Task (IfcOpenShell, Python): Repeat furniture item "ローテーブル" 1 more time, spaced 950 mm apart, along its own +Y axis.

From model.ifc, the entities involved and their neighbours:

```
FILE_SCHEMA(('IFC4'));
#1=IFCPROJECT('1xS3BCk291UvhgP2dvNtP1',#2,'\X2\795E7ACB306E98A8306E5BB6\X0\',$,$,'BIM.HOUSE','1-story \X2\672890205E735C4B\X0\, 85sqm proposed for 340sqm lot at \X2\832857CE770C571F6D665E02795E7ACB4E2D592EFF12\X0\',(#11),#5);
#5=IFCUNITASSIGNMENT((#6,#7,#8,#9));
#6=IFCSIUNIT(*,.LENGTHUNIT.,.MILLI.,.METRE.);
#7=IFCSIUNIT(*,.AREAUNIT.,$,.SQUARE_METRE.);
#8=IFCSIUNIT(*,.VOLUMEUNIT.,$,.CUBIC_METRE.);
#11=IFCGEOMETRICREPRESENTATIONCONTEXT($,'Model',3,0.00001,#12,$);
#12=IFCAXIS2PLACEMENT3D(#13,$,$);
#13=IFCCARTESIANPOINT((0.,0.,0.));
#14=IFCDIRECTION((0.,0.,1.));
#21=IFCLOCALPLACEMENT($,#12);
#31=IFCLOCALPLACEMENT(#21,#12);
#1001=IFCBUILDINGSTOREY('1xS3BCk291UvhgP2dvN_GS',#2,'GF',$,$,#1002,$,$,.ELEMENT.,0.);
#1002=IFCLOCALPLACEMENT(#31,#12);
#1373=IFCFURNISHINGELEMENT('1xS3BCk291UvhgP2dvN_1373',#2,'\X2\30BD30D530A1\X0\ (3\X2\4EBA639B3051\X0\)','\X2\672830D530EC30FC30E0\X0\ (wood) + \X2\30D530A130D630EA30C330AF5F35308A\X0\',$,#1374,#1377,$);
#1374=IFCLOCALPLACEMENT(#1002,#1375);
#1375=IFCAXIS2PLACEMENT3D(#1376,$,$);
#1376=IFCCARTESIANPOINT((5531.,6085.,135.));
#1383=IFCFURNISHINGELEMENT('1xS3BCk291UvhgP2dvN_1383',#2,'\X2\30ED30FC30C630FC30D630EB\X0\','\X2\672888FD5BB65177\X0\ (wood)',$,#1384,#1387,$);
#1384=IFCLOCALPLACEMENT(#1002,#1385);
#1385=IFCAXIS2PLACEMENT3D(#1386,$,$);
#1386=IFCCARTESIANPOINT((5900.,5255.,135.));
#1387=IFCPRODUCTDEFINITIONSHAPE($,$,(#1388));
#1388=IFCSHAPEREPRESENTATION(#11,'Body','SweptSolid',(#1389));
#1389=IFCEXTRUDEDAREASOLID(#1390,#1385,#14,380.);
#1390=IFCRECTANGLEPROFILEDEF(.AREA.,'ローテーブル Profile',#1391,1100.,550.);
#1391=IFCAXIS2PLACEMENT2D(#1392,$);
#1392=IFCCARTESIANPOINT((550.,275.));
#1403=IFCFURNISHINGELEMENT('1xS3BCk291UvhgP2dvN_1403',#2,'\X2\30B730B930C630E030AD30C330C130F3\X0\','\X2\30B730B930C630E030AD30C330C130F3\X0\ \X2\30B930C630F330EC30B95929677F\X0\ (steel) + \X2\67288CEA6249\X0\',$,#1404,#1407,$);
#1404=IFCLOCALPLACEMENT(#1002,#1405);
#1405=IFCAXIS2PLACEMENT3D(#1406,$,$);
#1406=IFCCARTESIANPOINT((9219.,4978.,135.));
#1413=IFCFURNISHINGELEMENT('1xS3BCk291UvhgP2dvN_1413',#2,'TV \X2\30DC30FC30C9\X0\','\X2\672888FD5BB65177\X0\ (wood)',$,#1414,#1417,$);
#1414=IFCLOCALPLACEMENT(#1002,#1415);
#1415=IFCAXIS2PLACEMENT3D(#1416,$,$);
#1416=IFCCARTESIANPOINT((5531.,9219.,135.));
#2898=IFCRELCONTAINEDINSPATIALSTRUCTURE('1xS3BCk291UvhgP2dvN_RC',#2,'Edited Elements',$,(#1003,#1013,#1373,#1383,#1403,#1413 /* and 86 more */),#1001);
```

```python
import ifcopenshell
import ifcopenshell.api.geometry
import ifcopenshell.api.root
import ifcopenshell.util.element
import ifcopenshell.util.placement

model = ifcopenshell.open("model.ifc")


def reuse_history(source, copy):
    """copy_class also copies each property set's owner history, people and application; keep the originals."""
    for rel in copy.IsDefinedBy:
        if rel.is_a("IfcRelDefinesByProperties") and (history := rel.RelatingPropertyDefinition.OwnerHistory):
            rel.RelatingPropertyDefinition.OwnerHistory = source.OwnerHistory
            ifcopenshell.util.element.remove_deep2(model, history)


source = model.by_id(1383)
base = ifcopenshell.util.placement.get_local_placement(source.ObjectPlacement)
step = base[:3, 1] * 950.0

for i in range(1, 2):
    copy = ifcopenshell.api.root.copy_class(model, product=source)
    copy.Representation = ifcopenshell.util.element.copy_deep(
        model, source.Representation, exclude=["IfcGeometricRepresentationContext", "IfcRepresentationMap"]
    )
    reuse_history(source, copy)
    matrix = base.copy()
    matrix[:3, 3] += i * step
    print("added at", matrix[:3, 3].round(3) + 0.0)
    ifcopenshell.api.geometry.edit_object_placement(model, product=copy, matrix=matrix, is_si=False)

model.write("model_updated.ifc")
```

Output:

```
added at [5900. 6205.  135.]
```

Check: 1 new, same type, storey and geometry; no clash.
